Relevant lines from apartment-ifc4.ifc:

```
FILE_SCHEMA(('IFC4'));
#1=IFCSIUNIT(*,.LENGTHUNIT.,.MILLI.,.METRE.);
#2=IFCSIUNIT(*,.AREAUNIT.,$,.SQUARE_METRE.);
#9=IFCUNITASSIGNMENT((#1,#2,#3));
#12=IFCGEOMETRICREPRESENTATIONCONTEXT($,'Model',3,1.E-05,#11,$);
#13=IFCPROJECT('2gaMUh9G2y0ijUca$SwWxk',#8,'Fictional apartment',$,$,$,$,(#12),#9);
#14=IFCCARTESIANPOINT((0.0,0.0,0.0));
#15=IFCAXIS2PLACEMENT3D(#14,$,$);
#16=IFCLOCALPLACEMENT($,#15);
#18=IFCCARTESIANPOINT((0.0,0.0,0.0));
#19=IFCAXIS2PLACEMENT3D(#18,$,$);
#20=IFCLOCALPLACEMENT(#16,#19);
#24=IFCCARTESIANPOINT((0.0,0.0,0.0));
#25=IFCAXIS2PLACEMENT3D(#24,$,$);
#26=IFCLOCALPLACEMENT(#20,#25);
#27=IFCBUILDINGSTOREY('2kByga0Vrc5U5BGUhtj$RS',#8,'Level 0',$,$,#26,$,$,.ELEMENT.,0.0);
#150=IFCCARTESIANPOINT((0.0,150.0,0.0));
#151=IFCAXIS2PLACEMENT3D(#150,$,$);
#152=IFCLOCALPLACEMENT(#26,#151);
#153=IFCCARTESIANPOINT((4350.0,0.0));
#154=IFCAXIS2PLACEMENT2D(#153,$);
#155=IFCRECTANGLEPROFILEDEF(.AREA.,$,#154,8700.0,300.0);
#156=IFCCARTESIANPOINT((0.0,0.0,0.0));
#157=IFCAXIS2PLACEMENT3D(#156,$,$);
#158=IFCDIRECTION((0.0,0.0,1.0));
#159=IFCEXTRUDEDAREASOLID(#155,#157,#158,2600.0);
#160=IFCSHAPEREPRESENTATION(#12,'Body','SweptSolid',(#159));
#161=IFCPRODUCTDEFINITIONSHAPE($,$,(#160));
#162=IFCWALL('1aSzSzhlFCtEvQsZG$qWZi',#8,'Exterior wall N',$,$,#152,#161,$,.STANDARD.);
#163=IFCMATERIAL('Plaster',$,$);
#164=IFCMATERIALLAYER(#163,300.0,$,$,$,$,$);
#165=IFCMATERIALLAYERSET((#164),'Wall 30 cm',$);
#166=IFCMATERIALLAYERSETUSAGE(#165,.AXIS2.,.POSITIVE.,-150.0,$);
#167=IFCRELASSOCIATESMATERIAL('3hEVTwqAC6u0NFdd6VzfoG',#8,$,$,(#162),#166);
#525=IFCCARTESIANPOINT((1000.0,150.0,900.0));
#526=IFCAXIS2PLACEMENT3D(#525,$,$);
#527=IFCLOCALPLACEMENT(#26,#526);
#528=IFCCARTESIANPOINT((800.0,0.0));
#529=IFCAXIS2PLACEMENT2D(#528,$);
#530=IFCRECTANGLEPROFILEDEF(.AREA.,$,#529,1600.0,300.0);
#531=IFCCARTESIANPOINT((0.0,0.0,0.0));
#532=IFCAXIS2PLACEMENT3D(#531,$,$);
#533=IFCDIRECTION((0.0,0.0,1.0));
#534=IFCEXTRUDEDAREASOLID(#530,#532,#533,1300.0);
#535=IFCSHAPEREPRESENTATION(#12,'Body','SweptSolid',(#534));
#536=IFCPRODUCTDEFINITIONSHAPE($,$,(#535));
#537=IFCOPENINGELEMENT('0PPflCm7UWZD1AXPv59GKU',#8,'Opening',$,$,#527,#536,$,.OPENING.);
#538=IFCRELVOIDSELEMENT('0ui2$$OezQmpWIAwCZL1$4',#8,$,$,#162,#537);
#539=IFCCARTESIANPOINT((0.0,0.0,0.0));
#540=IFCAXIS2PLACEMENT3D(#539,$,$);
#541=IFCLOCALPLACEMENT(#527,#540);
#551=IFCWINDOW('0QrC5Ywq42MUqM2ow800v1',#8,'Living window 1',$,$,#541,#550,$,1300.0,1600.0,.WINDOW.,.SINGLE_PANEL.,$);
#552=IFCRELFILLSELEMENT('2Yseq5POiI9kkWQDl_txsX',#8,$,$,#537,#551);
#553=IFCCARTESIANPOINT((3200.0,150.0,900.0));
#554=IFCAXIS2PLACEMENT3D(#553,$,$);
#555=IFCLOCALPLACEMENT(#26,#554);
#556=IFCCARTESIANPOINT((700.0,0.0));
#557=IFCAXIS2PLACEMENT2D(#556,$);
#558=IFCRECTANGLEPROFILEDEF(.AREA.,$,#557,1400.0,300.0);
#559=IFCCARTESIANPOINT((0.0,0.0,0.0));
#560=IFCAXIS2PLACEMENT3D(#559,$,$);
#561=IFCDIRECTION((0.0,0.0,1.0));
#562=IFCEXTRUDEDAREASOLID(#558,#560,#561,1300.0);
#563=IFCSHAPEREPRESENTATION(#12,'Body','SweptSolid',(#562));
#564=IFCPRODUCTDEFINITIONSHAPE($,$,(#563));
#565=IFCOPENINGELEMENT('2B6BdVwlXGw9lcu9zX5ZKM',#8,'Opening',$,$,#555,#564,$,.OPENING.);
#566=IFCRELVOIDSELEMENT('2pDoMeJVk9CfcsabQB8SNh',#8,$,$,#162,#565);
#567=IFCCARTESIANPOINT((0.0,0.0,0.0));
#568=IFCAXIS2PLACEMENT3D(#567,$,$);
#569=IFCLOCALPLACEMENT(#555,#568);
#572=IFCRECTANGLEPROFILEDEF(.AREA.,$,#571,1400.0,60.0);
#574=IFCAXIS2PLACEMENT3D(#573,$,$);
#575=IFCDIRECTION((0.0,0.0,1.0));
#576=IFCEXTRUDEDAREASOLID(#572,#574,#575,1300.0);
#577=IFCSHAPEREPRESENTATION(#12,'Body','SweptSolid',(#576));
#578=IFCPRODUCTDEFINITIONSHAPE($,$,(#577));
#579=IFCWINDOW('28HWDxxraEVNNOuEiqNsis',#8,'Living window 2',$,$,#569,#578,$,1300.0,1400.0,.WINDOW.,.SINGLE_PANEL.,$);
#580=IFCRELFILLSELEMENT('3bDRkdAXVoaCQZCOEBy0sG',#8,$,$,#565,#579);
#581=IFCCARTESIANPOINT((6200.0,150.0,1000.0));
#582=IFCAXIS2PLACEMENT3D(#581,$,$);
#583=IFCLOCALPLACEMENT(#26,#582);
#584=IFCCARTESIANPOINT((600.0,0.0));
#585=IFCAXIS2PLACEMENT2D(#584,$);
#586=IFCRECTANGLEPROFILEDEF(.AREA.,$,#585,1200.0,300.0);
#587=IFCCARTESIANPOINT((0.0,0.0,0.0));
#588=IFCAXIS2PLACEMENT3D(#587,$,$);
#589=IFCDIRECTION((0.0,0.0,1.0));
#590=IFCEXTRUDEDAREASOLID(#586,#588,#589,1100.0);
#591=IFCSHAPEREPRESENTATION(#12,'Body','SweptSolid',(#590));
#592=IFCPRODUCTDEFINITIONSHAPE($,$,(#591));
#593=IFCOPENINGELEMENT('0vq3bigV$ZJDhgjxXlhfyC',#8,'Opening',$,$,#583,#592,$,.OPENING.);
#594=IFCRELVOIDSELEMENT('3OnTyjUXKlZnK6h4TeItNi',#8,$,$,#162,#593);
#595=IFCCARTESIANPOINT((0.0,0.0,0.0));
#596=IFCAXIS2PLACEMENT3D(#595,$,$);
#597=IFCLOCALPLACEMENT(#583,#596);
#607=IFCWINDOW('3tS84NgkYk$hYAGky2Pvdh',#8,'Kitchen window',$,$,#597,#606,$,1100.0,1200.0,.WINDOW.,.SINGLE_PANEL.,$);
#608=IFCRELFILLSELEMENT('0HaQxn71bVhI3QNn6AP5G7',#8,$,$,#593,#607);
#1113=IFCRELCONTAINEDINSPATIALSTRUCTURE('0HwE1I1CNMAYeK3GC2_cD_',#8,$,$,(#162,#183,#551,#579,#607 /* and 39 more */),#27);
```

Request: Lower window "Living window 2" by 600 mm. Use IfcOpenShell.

```python
import numpy as np
import ifcopenshell
import ifcopenshell.api.geometry
import ifcopenshell.util.placement
import ifcopenshell.util.unit

model = ifcopenshell.open("apartment-ifc4.ifc")
unit_scale = ifcopenshell.util.unit.calculate_unit_scale(model)

window = model.by_guid("28HWDxxraEVNNOuEiqNsis")
opening = window.FillsVoids[0].RelatingOpeningElement
dz = -0.6 / unit_scale

shift = np.array([0.0, 0.0, dz])
# The window is placed relative to its opening, so it follows when the opening moves.
matrix = ifcopenshell.util.placement.get_local_placement(opening.ObjectPlacement)
matrix[:3, 3] += shift
ifcopenshell.api.geometry.edit_object_placement(
    model, product=opening, matrix=matrix, is_si=False, should_transform_children=True
)

print(f"moved by {dz * unit_scale:+.3f} m")

model.write("apartment-ifc4_edited.ifc")
```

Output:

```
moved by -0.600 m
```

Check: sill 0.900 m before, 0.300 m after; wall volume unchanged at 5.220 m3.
